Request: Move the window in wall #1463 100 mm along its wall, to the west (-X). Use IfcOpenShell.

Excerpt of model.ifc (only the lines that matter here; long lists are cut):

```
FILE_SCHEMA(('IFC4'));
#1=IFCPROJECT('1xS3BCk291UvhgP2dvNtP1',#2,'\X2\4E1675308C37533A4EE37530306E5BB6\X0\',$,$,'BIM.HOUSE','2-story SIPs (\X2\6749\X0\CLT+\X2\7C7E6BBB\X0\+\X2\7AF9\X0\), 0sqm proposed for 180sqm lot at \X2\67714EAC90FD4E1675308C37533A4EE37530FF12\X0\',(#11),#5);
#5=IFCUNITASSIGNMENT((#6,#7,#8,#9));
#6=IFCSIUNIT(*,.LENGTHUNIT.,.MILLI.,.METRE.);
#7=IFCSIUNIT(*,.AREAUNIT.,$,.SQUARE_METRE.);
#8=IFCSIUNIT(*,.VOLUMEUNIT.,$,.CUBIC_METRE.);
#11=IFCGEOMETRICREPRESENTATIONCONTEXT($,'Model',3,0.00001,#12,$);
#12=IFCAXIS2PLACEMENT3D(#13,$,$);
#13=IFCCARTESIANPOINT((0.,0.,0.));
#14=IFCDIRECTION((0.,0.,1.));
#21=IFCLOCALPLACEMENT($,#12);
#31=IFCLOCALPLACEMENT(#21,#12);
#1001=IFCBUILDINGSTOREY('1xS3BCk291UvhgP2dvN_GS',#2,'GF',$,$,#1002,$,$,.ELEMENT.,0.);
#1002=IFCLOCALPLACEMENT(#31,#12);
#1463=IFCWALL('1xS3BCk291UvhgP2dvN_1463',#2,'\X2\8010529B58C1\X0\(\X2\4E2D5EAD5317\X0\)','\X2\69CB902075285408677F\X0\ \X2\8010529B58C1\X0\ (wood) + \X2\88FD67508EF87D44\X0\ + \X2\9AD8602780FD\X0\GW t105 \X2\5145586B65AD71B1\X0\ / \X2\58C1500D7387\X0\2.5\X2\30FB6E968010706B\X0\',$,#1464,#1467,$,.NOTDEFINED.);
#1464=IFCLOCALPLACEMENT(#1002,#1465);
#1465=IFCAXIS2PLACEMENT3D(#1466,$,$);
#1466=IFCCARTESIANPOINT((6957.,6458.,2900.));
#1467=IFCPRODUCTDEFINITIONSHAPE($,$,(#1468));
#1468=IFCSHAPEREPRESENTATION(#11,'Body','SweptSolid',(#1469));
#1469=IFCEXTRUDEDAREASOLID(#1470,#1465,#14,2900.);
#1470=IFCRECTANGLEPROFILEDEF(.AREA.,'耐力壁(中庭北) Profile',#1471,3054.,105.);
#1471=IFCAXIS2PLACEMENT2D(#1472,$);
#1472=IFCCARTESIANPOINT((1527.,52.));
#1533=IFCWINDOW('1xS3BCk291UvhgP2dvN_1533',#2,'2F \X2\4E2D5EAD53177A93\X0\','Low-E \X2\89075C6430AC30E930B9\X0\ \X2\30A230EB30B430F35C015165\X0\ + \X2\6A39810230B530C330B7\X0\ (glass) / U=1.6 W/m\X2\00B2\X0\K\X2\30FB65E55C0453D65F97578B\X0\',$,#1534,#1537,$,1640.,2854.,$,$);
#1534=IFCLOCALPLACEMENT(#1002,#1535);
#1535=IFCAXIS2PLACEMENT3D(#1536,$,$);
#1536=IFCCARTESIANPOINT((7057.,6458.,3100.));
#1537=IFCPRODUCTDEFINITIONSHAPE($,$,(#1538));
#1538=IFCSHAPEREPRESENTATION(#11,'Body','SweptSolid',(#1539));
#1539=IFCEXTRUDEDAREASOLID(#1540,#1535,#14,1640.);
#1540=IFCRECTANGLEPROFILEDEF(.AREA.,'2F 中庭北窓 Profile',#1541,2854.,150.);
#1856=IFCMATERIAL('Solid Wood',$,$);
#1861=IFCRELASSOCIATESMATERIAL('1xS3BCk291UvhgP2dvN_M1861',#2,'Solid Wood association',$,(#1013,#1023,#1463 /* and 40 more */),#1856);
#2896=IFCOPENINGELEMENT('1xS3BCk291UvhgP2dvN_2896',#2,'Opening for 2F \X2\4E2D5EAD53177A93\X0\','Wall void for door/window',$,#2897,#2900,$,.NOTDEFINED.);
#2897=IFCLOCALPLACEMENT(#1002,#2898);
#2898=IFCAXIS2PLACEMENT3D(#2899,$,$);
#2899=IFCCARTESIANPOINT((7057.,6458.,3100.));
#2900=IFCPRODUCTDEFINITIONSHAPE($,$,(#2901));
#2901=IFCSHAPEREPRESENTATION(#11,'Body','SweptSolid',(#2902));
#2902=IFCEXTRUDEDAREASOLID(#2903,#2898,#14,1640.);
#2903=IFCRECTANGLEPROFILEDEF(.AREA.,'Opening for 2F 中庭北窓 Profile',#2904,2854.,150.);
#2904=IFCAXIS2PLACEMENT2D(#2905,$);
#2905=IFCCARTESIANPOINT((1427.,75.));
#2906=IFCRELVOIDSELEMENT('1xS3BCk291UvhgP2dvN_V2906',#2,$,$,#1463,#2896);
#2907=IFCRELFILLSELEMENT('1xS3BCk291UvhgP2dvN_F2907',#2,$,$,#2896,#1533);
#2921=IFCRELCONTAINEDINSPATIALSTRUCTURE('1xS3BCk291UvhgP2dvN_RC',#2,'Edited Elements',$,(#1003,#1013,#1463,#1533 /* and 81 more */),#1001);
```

```python
import ifcopenshell
import ifcopenshell.api.geometry
import ifcopenshell.util.placement

model = ifcopenshell.open("model.ifc")

window = model.by_guid("1xS3BCk291UvhgP2dvN_1533")
opening = window.FillsVoids[0].RelatingOpeningElement
wall = opening.VoidsElements[0].RelatingBuildingElement

wall_matrix = ifcopenshell.util.placement.get_local_placement(wall.ObjectPlacement)
shift = wall_matrix[:3, 0] * -100.0
before = ifcopenshell.util.placement.get_local_placement(window.ObjectPlacement)[:3, 3].copy()

# The window is not placed relative to its opening, so move both.
for product in (opening, window):
    matrix = ifcopenshell.util.placement.get_local_placement(product.ObjectPlacement)
    matrix[:3, 3] += shift
    ifcopenshell.api.geometry.edit_object_placement(model, product=product, matrix=matrix, is_si=False)

after = ifcopenshell.util.placement.get_local_placement(window.ObjectPlacement)[:3, 3]
print("window moved by", (after - before).round(3) + 0.0)

model.write("model_edited.ifc")
```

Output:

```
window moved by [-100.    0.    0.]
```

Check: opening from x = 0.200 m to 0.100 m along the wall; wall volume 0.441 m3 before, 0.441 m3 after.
